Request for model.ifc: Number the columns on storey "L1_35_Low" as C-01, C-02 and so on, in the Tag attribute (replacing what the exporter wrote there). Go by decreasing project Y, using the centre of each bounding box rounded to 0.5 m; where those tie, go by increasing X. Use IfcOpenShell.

First a look at what the model holds.

```python
import ifcopenshell
import ifcopenshell.util.element
import ifcopenshell.util.placement

model = ifcopenshell.open("model.ifc")
print(model.schema)
storey = next(s for s in model.by_type("IfcBuildingStorey") if s.Name == "L1_35_Low")
columns = [e for e in ifcopenshell.util.element.get_decomposition(storey) if e.is_a("IfcColumn")]
for e in sorted(columns, key=lambda e: e.id()):
    origin = ifcopenshell.util.placement.get_local_placement(e.ObjectPlacement)[:3, 3]
    print(e.id(), e.Tag, e.Name, origin.round(2) + 0.0, sep=" | ")
```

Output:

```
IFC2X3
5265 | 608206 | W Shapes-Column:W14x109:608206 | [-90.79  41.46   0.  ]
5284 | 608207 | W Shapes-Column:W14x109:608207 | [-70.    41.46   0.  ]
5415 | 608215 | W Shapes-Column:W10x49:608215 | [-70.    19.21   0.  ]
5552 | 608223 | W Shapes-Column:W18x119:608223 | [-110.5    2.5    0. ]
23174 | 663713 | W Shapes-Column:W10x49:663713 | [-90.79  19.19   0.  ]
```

```python
import ifcopenshell
import ifcopenshell.geom
import ifcopenshell.util.element
import ifcopenshell.util.shape

model = ifcopenshell.open("model.ifc")
settings = ifcopenshell.geom.settings()
settings.set("use-world-coords", True)


def centre(element):
    shape = ifcopenshell.geom.create_shape(settings, element)
    return ifcopenshell.util.shape.get_bbox_centroid(shape.geometry)


storey = next(s for s in model.by_type("IfcBuildingStorey") if s.Name == "L1_35_Low")
columns = [e for e in ifcopenshell.util.element.get_decomposition(storey) if e.is_a("IfcColumn")]

# Insertion points can sit at a corner or the storey origin, so sort by the geometry (in metres).
centres = {e: centre(e) for e in columns}
columns.sort(key=lambda e: (-round(centres[e][1] / 0.5), centres[e][0]))

for i, e in enumerate(columns, start=1):
    number = f"C-{i:02d}"
    e.Tag = number
    print(e.id(), number)

model.write("model_updated.ifc")
```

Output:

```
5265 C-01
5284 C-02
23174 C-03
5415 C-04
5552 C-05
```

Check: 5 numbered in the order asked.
